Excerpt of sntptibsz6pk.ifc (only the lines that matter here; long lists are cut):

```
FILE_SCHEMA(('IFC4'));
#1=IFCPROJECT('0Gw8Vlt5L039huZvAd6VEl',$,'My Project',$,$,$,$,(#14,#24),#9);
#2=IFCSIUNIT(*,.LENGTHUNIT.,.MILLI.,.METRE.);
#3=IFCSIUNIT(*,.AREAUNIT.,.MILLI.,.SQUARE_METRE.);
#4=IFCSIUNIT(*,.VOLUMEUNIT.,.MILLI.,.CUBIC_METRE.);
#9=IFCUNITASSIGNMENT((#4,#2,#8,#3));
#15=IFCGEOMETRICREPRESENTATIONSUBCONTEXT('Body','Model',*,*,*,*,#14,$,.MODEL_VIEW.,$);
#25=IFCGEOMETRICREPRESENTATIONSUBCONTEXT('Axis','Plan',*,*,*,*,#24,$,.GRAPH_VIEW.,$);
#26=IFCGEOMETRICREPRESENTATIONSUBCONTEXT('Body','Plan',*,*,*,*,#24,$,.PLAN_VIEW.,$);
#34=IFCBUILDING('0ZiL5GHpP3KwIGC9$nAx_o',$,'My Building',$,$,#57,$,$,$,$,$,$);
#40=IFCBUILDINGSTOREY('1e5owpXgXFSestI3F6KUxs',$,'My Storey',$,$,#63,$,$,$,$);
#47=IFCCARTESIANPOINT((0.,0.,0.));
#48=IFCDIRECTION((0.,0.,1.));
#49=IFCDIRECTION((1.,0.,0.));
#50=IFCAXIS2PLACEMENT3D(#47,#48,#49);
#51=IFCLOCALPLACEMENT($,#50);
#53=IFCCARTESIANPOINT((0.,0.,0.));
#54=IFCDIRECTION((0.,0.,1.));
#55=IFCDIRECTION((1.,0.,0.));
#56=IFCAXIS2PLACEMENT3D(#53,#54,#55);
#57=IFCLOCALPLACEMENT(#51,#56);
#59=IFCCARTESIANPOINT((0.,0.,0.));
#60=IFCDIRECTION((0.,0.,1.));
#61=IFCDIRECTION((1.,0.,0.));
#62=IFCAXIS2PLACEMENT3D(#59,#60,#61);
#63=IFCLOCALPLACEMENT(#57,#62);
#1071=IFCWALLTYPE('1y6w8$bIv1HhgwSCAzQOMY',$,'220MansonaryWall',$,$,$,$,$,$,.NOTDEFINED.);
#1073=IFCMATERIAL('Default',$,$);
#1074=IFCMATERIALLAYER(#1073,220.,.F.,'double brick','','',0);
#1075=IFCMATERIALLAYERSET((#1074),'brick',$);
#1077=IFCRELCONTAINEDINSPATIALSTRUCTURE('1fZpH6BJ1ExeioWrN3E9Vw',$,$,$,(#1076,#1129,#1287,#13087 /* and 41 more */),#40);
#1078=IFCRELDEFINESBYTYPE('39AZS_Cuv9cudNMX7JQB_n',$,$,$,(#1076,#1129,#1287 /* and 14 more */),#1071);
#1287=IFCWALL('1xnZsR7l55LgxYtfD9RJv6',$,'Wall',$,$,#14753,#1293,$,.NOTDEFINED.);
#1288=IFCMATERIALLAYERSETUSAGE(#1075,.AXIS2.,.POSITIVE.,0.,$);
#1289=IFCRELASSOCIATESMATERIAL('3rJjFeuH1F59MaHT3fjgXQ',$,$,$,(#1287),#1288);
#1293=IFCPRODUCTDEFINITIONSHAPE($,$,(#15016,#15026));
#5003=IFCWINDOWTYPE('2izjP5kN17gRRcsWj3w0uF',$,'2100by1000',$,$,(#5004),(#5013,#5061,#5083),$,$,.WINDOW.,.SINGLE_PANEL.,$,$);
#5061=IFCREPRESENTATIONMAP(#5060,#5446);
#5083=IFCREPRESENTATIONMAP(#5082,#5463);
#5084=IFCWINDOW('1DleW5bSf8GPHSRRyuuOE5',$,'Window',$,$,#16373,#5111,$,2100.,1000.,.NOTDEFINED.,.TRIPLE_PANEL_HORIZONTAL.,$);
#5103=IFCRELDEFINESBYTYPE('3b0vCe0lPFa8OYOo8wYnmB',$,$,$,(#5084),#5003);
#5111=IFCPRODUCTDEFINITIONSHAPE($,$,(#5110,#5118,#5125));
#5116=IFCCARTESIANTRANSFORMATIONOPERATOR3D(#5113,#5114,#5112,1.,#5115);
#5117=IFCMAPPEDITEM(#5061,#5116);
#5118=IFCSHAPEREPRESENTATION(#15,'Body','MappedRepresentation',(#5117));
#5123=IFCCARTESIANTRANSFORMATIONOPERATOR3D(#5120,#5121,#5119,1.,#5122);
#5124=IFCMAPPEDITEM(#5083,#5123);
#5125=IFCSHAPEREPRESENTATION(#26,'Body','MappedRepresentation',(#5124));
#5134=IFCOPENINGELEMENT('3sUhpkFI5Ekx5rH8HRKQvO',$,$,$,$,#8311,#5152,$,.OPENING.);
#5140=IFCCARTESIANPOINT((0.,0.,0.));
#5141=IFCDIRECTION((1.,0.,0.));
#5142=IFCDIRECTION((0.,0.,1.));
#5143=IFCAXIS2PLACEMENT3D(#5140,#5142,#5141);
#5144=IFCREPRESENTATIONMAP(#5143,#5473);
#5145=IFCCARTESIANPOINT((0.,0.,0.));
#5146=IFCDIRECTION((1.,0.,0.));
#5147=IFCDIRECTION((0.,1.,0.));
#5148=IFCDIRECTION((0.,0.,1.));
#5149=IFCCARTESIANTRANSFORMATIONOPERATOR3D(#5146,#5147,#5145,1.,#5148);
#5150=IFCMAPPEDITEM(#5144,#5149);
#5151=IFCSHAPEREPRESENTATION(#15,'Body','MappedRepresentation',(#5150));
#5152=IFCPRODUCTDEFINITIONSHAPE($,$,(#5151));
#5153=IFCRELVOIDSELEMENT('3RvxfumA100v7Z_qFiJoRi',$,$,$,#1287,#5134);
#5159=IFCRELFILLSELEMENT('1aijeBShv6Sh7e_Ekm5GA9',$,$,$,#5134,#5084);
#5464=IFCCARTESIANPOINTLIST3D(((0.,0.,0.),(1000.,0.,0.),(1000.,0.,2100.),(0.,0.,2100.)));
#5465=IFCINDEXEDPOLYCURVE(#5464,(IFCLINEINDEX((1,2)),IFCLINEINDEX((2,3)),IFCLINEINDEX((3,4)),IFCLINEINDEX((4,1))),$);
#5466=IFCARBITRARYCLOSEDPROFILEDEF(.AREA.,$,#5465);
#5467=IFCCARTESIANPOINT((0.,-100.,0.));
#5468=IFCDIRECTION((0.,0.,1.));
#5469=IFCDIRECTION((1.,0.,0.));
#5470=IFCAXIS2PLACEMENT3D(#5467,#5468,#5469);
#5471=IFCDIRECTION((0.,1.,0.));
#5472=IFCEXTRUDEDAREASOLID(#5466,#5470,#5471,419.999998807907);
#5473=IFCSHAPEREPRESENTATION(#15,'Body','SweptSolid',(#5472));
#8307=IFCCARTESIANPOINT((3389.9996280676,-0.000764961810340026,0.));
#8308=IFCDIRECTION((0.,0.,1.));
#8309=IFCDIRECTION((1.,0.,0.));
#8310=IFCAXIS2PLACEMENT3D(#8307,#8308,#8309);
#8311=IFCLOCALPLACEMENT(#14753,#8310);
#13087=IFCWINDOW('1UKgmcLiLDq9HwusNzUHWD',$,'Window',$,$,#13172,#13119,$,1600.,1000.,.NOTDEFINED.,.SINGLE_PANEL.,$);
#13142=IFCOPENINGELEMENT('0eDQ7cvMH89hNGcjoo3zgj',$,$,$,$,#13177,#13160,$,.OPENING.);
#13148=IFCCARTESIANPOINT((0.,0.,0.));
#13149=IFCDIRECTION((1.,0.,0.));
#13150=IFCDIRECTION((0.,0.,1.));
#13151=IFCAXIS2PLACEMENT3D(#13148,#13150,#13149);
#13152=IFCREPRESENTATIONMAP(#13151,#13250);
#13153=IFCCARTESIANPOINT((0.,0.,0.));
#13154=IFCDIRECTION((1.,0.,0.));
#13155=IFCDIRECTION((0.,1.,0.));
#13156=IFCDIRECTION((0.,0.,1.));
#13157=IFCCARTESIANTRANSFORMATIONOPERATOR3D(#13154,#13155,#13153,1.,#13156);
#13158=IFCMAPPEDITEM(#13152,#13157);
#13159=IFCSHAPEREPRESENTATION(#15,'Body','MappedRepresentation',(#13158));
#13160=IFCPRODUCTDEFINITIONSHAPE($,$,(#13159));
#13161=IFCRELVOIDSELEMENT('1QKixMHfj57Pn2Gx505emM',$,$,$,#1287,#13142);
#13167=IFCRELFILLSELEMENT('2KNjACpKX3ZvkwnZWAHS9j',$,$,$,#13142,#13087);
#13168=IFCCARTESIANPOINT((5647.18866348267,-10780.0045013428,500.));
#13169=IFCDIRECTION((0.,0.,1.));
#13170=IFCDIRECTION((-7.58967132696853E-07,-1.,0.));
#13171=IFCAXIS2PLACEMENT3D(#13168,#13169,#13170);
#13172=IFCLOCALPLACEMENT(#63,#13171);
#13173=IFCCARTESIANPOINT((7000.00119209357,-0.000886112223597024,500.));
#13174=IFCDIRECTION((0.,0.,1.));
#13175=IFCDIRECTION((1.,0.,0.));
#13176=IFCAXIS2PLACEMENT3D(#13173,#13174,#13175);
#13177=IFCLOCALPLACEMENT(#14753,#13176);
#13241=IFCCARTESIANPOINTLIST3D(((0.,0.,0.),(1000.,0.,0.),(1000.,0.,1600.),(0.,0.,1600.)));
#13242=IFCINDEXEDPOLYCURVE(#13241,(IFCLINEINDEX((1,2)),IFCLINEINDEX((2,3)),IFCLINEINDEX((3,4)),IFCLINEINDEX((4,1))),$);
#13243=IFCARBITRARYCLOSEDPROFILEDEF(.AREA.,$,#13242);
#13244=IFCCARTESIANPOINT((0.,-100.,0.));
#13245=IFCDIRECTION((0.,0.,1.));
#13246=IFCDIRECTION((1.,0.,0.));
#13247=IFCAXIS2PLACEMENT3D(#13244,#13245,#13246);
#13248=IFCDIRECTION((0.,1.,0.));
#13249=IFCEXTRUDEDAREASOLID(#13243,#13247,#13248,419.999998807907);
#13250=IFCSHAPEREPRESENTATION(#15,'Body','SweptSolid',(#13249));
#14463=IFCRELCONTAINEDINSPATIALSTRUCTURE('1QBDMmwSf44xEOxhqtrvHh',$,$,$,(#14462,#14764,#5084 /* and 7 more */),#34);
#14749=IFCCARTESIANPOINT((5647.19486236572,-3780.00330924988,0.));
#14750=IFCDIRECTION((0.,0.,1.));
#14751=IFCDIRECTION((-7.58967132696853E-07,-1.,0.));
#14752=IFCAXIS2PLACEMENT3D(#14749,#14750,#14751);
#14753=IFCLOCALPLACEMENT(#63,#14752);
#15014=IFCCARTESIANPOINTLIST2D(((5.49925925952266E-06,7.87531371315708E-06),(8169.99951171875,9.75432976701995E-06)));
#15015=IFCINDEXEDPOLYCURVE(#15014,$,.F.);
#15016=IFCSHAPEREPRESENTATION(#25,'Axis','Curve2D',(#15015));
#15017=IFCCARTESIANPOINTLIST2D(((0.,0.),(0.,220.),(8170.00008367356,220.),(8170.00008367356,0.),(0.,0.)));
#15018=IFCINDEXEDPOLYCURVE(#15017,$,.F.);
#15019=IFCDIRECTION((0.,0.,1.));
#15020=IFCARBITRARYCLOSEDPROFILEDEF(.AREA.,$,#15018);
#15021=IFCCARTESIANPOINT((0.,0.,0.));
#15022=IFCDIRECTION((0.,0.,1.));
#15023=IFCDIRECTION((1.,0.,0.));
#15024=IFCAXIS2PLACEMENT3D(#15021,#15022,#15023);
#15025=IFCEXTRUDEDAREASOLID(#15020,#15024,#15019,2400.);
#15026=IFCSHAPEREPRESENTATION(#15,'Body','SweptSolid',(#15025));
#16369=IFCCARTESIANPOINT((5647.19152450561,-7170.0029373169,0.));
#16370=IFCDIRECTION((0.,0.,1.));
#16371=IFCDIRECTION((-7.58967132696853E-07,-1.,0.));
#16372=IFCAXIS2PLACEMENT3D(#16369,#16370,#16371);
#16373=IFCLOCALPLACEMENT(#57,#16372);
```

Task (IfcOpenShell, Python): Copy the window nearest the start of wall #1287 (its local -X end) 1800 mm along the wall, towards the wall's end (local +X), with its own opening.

```python
import ifcopenshell
import ifcopenshell.api.feature
import ifcopenshell.api.geometry
import ifcopenshell.api.root
import ifcopenshell.geom
import ifcopenshell.util.element
import ifcopenshell.util.placement
import ifcopenshell.util.shape
import ifcopenshell.util.unit

model = ifcopenshell.open("sntptibsz6pk.ifc")
unit_scale = ifcopenshell.util.unit.calculate_unit_scale(model)
settings = ifcopenshell.geom.settings()


def volume(element):
    """Net volume in cubic metres, openings subtracted."""
    shape = ifcopenshell.geom.create_shape(settings, element)
    return ifcopenshell.util.shape.get_volume(shape.geometry)


window = model.by_guid("1DleW5bSf8GPHSRRyuuOE5")
opening = window.FillsVoids[0].RelatingOpeningElement
wall = opening.VoidsElements[0].RelatingBuildingElement
before = volume(wall)
shift = ifcopenshell.util.placement.get_local_placement(wall.ObjectPlacement)[:3, 0] * 1.8 / unit_scale

# copy_class copies the void relationship, type, container and properties, but no geometry.
new_opening = ifcopenshell.api.root.copy_class(model, product=opening)
new_opening.Representation = ifcopenshell.util.element.copy_deep(
    model, opening.Representation, exclude=["IfcGeometricRepresentationContext", "IfcRepresentationMap"]
)
new_window = ifcopenshell.api.root.copy_class(model, product=window)
new_window.Representation = ifcopenshell.util.element.copy_deep(
    model, window.Representation, exclude=["IfcGeometricRepresentationContext", "IfcRepresentationMap"]
)
ifcopenshell.api.feature.add_filling(model, opening=new_opening, element=new_window)

for old, new in ((opening, new_opening), (window, new_window)):
    matrix = ifcopenshell.util.placement.get_local_placement(old.ObjectPlacement)
    matrix[:3, 3] += shift
    ifcopenshell.api.geometry.edit_object_placement(model, product=new, matrix=matrix, is_si=False)

after = volume(wall)

print(f"wall volume {before:.3f} -> {after:.3f} m3")

model.write("sntptibsz6pk_v2.ifc")
```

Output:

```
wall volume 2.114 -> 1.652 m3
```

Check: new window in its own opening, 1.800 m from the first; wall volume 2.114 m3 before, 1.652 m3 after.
